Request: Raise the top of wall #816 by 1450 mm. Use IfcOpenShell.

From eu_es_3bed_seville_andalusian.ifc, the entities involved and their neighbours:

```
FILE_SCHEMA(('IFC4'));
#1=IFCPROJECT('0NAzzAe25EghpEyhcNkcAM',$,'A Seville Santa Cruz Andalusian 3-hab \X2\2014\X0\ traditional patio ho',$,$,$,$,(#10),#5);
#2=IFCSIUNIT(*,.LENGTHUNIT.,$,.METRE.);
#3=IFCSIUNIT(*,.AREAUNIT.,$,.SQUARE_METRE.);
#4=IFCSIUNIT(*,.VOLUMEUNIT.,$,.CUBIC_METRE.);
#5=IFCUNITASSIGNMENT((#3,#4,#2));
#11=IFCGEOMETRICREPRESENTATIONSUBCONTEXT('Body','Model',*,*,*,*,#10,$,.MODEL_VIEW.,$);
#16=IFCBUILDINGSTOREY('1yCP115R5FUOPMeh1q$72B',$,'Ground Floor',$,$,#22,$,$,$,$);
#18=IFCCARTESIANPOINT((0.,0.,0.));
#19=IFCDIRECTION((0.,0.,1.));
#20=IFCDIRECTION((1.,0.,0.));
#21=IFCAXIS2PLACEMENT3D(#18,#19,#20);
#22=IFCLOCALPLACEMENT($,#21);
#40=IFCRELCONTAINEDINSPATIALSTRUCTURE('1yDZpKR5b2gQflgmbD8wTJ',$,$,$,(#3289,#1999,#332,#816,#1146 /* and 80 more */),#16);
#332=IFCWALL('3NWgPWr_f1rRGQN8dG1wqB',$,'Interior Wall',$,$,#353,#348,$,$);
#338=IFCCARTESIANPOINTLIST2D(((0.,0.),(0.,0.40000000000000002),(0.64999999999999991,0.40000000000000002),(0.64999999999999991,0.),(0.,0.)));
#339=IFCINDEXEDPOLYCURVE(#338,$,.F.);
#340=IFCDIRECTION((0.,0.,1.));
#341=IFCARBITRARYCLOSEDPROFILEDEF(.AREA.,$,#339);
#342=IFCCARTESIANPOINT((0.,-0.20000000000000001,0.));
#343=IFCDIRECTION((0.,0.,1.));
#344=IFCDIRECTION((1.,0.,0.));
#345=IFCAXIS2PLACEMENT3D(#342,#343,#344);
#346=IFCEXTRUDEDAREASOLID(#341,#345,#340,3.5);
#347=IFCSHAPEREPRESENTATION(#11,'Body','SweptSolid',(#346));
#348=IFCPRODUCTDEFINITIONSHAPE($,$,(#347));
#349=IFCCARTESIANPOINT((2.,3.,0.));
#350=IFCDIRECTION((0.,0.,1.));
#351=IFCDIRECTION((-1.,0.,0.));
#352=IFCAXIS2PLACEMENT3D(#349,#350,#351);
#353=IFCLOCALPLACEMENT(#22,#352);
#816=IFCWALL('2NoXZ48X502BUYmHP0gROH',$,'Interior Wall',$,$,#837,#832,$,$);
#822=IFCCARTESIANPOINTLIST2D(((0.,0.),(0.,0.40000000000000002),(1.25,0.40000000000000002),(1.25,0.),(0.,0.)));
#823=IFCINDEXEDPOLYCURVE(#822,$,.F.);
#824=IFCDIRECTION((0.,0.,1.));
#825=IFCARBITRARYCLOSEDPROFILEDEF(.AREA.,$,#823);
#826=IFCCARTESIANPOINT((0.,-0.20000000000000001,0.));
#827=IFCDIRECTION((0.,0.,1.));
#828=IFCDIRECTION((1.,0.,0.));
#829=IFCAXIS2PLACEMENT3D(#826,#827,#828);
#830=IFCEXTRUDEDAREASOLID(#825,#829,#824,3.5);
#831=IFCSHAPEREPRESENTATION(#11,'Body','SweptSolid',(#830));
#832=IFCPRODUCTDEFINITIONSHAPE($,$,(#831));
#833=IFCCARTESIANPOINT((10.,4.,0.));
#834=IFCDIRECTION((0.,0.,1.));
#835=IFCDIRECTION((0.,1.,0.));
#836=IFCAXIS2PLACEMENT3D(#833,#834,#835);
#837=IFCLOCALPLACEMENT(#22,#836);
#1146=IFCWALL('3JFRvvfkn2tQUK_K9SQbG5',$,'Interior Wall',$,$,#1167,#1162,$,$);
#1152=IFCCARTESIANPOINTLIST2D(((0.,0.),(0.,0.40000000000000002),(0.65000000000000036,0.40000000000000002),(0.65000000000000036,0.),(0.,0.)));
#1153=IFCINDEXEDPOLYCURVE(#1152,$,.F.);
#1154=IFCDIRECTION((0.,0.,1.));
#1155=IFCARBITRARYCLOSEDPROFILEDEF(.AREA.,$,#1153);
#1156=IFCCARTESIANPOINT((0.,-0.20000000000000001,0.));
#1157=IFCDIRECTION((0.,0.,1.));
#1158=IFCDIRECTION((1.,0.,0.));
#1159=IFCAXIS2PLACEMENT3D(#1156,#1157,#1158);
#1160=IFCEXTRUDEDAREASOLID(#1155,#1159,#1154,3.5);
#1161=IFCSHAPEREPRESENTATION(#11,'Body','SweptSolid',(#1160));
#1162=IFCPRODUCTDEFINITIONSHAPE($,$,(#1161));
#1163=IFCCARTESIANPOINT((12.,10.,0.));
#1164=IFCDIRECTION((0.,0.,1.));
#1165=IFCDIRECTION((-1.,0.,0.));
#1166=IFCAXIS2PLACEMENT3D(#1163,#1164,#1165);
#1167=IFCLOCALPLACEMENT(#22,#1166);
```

```python
import ifcopenshell
import ifcopenshell.geom
import ifcopenshell.util.representation
import ifcopenshell.util.shape

model = ifcopenshell.open("eu_es_3bed_seville_andalusian.ifc")
settings = ifcopenshell.geom.settings()


def volume(element):
    """Net volume in cubic metres, openings subtracted."""
    shape = ifcopenshell.geom.create_shape(settings, element)
    return ifcopenshell.util.shape.get_volume(shape.geometry)


wall = model.by_id(816)
before = volume(wall)

body = ifcopenshell.util.representation.get_representation(wall, "Model", "Body")
solid = body.Items[0]
old_height = solid.Depth
solid.Depth += 1.45
after = volume(wall)

print(f"height {old_height:g} -> {solid.Depth:g}, volume {before:.3f} -> {after:.3f} m3")

model.write("eu_es_3bed_seville_andalusian_v2.ifc")
```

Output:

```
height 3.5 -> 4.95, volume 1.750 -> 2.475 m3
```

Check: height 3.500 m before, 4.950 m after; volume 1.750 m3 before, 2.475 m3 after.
